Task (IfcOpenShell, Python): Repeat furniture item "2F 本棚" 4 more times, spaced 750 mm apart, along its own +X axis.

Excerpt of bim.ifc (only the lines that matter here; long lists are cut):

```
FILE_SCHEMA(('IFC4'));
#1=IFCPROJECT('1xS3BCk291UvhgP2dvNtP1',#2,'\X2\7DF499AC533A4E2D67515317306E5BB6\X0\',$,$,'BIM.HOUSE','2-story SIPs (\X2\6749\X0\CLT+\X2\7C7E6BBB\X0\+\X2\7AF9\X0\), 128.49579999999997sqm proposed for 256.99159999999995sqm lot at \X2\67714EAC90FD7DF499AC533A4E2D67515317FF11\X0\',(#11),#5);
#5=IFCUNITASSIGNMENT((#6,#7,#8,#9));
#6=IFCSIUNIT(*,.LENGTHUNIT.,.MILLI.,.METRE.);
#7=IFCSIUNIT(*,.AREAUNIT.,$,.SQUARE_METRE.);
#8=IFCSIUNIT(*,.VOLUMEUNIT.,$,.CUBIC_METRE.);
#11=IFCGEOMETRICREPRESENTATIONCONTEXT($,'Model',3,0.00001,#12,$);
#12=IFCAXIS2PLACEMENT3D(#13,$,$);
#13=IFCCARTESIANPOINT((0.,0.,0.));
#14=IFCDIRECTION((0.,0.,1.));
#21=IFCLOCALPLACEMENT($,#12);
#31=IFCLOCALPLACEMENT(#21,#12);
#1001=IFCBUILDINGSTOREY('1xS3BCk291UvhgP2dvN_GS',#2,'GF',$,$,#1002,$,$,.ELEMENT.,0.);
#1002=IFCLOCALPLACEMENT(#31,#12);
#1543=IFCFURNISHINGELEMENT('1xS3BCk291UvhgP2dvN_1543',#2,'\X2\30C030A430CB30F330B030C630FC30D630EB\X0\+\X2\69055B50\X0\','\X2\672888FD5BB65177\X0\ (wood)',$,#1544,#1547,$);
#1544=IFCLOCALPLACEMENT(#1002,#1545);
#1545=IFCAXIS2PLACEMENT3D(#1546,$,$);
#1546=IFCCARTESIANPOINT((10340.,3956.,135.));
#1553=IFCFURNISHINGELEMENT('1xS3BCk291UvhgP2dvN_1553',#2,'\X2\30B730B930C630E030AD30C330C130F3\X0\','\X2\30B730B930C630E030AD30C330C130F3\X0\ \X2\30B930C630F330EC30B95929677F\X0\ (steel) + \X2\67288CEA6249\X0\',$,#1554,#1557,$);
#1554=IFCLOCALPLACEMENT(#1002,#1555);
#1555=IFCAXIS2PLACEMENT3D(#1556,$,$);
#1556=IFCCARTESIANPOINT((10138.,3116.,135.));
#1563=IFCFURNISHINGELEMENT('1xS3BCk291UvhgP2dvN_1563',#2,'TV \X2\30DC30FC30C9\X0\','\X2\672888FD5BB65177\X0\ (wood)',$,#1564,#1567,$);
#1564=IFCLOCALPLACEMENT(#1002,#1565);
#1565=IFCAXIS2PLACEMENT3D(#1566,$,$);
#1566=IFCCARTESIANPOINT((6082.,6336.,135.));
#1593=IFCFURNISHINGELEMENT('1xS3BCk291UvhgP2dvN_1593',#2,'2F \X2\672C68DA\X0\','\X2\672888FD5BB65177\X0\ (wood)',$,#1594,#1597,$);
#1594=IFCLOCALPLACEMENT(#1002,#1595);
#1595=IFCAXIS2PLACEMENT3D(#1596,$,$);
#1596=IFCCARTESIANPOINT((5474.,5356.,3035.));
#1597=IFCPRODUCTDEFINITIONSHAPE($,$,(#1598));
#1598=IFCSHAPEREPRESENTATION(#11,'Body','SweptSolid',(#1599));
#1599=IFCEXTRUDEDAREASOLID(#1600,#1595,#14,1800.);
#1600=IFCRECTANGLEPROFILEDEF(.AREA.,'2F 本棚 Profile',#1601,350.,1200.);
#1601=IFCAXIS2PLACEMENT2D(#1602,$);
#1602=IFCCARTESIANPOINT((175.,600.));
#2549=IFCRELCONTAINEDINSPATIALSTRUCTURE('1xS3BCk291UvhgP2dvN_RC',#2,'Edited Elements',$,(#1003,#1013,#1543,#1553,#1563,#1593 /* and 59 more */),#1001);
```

```python
import ifcopenshell
import ifcopenshell.api.geometry
import ifcopenshell.api.root
import ifcopenshell.util.element
import ifcopenshell.util.placement

model = ifcopenshell.open("bim.ifc")


def reuse_history(source, copy):
    """copy_class also copies each property set's owner history, people and application; keep the originals."""
    for rel in copy.IsDefinedBy:
        if rel.is_a("IfcRelDefinesByProperties") and (history := rel.RelatingPropertyDefinition.OwnerHistory):
            rel.RelatingPropertyDefinition.OwnerHistory = source.OwnerHistory
            ifcopenshell.util.element.remove_deep2(model, history)


source = model.by_guid("1xS3BCk291UvhgP2dvN_1593")
base = ifcopenshell.util.placement.get_local_placement(source.ObjectPlacement)
step = base[:3, 0] * 750.0

for i in range(1, 5):
    copy = ifcopenshell.api.root.copy_class(model, product=source)
    copy.Representation = ifcopenshell.util.element.copy_deep(
        model, source.Representation, exclude=["IfcGeometricRepresentationContext", "IfcRepresentationMap"]
    )
    reuse_history(source, copy)
    matrix = base.copy()
    matrix[:3, 3] += i * step
    print("added at", matrix[:3, 3].round(3) + 0.0)
    ifcopenshell.api.geometry.edit_object_placement(model, product=copy, matrix=matrix, is_si=False)

model.write("bim_edited.ifc")
```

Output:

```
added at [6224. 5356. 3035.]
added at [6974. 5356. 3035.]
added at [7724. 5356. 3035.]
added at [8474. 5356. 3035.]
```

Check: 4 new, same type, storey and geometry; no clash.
